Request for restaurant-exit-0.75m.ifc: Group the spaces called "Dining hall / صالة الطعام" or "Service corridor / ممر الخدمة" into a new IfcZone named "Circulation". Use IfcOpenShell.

First a look at what the model holds.

```python
import ifcopenshell

model = ifcopenshell.open("restaurant-exit-0.75m.ifc")
print(model.schema)
seen = {}
for space in model.by_type("IfcSpace"):
    seen[space.LongName] = seen.get(space.LongName, 0) + 1
for name, count in sorted(seen.items(), key=str):
    print(count, "x", name)
print("zones:", [z.Name for z in model.by_type("IfcZone")][:20])
```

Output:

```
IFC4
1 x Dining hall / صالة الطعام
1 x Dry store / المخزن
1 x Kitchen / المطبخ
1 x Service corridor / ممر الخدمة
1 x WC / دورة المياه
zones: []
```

```python
import ifcopenshell
import ifcopenshell.api.group
import ifcopenshell.api.root

model = ifcopenshell.open("restaurant-exit-0.75m.ifc")

names = {"Dining hall / صالة الطعام", "Service corridor / ممر الخدمة"}
spaces = [s for s in model.by_type("IfcSpace") if s.LongName in names]

zone = ifcopenshell.api.root.create_entity(model, ifc_class="IfcZone", name="Circulation")
ifcopenshell.api.group.assign_group(model, products=spaces, group=zone)
print(len(spaces), "spaces in", zone.Name)

model.write("restaurant-exit-0.75m-out.ifc")
```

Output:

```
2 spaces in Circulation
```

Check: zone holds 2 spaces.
